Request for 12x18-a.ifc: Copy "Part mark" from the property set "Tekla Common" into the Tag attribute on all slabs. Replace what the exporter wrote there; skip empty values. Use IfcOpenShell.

First a look at what the model holds.

```python
import ifcopenshell
import ifcopenshell.util.element

model = ifcopenshell.open("12x18-a.ifc")
print(model.schema)
slabs = model.by_type("IfcSlab")
print(len(slabs), "slabs")
for e in slabs[:8]:
    source = ifcopenshell.util.element.get_pset(e, "Tekla Common", "Part mark")
    target = e.Tag
    print(e.id(), repr(source), repr(target), sep=" | ")
```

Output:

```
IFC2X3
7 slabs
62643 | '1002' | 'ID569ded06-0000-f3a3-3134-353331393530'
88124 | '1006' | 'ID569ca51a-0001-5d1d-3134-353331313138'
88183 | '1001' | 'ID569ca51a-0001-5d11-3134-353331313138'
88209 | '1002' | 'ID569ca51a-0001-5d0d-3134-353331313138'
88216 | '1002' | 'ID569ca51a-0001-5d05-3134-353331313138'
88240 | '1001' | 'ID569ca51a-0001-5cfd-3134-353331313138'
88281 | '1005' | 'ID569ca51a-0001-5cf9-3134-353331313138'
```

```python
import ifcopenshell
import ifcopenshell.util.element

model = ifcopenshell.open("12x18-a.ifc")

count = 0
for e in model.by_type("IfcSlab"):
    value = ifcopenshell.util.element.get_pset(e, "Tekla Common", "Part mark")
    current = e.Tag
    if not value or not value.strip() or current == value:
        continue
    e.Tag = value
    count += 1

print(count, "slabs updated")

model.write("12x18-a-out.ifc")
```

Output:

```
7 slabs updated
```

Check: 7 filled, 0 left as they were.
